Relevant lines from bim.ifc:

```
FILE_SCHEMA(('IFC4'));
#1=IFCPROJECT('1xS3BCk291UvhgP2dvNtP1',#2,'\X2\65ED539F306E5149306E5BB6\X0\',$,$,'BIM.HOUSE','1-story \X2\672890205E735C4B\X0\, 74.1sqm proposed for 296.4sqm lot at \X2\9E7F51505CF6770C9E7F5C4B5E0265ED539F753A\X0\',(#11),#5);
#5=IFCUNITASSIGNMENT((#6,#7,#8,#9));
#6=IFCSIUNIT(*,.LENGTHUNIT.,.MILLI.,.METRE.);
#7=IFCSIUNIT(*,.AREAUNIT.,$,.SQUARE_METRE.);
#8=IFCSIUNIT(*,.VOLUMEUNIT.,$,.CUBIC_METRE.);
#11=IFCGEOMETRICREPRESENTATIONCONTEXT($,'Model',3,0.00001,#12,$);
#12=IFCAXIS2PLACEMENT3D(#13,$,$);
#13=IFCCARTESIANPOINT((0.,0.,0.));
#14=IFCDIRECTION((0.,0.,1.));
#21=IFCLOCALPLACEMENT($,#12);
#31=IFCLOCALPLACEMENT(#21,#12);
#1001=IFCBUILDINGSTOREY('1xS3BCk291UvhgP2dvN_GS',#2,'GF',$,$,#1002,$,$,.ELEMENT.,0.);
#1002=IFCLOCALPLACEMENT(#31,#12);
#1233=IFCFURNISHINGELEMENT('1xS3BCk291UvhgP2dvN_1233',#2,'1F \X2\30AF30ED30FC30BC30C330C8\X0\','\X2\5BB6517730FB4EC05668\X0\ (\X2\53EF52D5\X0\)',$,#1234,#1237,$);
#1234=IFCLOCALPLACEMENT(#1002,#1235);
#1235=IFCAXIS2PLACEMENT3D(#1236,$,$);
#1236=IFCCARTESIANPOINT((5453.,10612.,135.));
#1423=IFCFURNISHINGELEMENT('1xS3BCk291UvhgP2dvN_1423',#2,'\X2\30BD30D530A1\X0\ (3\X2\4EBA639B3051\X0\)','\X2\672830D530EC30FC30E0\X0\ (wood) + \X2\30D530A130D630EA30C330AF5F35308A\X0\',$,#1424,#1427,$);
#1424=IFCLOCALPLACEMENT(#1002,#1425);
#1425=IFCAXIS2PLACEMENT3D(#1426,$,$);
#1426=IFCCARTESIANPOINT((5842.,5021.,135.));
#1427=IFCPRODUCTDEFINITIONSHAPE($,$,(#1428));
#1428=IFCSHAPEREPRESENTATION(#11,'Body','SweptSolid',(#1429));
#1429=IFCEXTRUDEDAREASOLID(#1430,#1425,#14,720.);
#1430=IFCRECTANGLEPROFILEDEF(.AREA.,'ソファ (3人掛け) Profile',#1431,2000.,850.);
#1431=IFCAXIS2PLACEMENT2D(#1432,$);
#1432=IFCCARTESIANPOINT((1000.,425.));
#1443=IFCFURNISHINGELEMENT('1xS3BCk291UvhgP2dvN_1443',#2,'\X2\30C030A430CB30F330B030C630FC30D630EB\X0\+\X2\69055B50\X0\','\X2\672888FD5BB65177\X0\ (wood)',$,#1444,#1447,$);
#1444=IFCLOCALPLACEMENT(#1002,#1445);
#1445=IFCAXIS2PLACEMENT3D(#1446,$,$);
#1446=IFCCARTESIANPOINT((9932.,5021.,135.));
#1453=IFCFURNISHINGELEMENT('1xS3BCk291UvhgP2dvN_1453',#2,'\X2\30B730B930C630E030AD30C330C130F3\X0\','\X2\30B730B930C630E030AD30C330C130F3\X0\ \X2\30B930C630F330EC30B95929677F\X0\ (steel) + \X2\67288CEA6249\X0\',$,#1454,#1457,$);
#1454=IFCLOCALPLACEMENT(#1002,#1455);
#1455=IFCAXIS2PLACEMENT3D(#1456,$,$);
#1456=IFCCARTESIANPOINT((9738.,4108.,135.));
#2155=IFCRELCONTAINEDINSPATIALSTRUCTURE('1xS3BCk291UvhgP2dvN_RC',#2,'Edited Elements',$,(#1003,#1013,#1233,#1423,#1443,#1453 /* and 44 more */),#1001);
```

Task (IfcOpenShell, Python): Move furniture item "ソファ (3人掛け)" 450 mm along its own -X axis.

```python
import ifcopenshell
import ifcopenshell.api.geometry
import ifcopenshell.util.placement
import ifcopenshell.util.unit

model = ifcopenshell.open("bim.ifc")
unit_scale = ifcopenshell.util.unit.calculate_unit_scale(model)

item = model.by_guid("1xS3BCk291UvhgP2dvN_1423")
matrix = ifcopenshell.util.placement.get_local_placement(item.ObjectPlacement)
matrix[:3, 3] -= matrix[:3, 0] * 0.45 / unit_scale
ifcopenshell.api.geometry.edit_object_placement(model, product=item, matrix=matrix, is_si=False)

print(ifcopenshell.util.placement.get_local_placement(item.ObjectPlacement).round(3) + 0.0)

model.write("bim_v2.ifc")
```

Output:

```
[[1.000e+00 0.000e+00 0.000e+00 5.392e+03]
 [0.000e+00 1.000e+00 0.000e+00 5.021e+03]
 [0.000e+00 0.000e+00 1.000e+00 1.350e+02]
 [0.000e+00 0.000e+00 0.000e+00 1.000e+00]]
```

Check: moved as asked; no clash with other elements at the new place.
